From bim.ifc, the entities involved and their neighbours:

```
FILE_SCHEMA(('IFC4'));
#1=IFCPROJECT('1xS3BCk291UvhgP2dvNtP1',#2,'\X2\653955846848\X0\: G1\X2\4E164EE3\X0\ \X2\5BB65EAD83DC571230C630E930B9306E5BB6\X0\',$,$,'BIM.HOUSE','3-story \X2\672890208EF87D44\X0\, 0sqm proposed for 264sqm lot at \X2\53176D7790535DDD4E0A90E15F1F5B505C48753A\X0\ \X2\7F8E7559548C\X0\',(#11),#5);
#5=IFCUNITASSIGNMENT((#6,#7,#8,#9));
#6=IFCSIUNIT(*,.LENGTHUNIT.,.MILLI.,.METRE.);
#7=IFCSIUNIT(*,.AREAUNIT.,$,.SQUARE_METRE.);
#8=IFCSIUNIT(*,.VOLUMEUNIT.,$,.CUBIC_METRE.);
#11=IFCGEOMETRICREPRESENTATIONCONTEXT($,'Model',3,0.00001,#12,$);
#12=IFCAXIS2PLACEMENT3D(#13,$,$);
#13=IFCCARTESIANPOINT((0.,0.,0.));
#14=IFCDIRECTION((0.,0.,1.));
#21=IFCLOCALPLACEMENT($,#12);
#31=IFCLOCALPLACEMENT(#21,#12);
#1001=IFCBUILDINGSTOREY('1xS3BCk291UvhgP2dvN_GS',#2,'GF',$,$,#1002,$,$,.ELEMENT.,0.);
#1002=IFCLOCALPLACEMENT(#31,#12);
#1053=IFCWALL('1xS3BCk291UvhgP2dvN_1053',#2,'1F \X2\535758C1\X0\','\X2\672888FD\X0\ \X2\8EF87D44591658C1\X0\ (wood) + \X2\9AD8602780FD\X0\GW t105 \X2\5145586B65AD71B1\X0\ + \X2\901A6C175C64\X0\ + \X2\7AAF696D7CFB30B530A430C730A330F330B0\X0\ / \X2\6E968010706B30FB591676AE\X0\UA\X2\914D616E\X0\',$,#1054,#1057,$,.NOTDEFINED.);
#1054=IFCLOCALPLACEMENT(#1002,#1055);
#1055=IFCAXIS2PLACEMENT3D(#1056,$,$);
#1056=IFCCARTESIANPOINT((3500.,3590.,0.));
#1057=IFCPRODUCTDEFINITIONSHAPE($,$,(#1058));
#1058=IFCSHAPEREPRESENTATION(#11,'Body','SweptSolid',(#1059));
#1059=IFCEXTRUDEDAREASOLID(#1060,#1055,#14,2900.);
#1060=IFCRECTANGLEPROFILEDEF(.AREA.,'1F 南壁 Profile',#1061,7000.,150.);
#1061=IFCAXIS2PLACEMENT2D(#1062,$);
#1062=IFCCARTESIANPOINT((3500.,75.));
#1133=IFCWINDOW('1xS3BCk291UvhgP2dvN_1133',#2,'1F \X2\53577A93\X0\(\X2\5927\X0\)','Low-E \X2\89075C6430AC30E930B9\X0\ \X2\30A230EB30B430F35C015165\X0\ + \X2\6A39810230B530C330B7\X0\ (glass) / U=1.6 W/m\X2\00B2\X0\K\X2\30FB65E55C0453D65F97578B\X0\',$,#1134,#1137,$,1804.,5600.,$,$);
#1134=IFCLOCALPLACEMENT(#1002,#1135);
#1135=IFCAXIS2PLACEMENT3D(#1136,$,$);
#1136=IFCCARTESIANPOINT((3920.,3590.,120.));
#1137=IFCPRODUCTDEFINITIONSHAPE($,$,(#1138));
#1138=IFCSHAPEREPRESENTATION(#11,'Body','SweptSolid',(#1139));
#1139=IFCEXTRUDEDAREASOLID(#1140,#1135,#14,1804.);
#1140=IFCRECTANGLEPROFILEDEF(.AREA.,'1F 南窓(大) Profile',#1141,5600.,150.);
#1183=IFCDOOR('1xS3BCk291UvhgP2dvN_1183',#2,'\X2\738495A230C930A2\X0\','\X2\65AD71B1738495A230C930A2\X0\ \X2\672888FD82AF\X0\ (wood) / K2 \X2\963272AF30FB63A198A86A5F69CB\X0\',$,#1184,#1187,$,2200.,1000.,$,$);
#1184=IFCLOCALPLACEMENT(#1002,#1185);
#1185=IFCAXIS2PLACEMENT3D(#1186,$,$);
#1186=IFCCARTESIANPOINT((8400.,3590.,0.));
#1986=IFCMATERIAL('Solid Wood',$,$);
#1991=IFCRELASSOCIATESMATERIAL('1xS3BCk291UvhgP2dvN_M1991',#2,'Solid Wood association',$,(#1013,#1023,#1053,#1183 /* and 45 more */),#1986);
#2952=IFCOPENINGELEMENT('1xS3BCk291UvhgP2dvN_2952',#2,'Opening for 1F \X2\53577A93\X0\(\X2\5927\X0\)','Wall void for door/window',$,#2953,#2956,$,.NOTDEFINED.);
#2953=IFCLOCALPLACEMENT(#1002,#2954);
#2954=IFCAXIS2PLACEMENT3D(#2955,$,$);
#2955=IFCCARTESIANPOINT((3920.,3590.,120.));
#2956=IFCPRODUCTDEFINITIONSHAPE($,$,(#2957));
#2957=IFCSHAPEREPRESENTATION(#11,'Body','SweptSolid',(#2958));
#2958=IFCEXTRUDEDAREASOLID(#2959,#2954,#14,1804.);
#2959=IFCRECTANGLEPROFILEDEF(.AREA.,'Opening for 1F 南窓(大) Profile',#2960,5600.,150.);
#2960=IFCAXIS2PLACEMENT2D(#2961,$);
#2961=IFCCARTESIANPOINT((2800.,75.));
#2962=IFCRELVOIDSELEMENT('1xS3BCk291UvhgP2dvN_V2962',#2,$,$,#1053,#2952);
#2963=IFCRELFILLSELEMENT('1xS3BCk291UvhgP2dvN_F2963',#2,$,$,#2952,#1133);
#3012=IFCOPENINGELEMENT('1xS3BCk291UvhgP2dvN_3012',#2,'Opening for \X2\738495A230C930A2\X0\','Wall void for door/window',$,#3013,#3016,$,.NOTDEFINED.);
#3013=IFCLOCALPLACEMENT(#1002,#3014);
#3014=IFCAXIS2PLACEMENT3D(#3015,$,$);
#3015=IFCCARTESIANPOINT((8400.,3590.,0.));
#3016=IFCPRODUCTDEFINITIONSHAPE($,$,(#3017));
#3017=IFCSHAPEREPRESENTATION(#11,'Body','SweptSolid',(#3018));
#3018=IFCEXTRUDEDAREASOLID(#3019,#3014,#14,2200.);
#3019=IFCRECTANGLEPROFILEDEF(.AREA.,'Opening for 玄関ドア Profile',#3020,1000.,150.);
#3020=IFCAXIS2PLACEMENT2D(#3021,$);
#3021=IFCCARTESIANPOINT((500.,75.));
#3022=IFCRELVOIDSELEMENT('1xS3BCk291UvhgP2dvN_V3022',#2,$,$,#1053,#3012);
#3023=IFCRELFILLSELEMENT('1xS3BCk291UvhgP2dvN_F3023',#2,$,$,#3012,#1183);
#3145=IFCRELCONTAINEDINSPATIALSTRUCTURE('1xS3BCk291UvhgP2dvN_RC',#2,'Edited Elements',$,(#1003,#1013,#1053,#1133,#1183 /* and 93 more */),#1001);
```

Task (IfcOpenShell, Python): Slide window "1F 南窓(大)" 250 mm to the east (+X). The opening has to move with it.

```python
import ifcopenshell
import ifcopenshell.api.geometry
import ifcopenshell.util.placement

model = ifcopenshell.open("bim.ifc")

window = model.by_guid("1xS3BCk291UvhgP2dvN_1133")
opening = window.FillsVoids[0].RelatingOpeningElement
wall = opening.VoidsElements[0].RelatingBuildingElement

wall_matrix = ifcopenshell.util.placement.get_local_placement(wall.ObjectPlacement)
shift = wall_matrix[:3, 0] * 250.0
before = ifcopenshell.util.placement.get_local_placement(window.ObjectPlacement)[:3, 3].copy()

# The window is not placed relative to its opening, so move both.
for product in (opening, window):
    matrix = ifcopenshell.util.placement.get_local_placement(product.ObjectPlacement)
    matrix[:3, 3] += shift
    ifcopenshell.api.geometry.edit_object_placement(model, product=product, matrix=matrix, is_si=False)

after = ifcopenshell.util.placement.get_local_placement(window.ObjectPlacement)[:3, 3]
print("window moved by", (after - before).round(3) + 0.0)

model.write("bim_v2.ifc")
```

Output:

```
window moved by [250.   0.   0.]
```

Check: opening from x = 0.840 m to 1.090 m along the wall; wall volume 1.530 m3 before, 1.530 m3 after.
